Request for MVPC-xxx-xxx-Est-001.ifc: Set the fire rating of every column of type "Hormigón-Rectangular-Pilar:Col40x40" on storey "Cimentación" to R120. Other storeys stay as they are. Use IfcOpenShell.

First a look at what the model holds.

```python
import ifcopenshell
import ifcopenshell.util.element

model = ifcopenshell.open("MVPC-xxx-xxx-Est-001.ifc")
print(model.schema)
storey = next(s for s in model.by_type("IfcBuildingStorey") if s.Name == "Cimentación")
columns = [e for e in ifcopenshell.util.element.get_decomposition(storey) if e.is_a("IfcColumn")]
seen = {}
for e in columns:
    element_type = ifcopenshell.util.element.get_type(e)
    key = (element_type.Name if element_type != e and element_type else None, ifcopenshell.util.element.get_pset(e, "Pset_ColumnCommon", "FireRating"))
    seen[key] = seen.get(key, 0) + 1
for (name, value), count in sorted(seen.items(), key=str):
    print(count, "x", name, "|", value)
```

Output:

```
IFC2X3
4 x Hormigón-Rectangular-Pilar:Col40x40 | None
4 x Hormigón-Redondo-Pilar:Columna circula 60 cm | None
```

```python
import ifcopenshell
import ifcopenshell.api.pset
import ifcopenshell.util.element

model = ifcopenshell.open("MVPC-xxx-xxx-Est-001.ifc")

storey = next(s for s in model.by_type("IfcBuildingStorey") if s.Name == "Cimentación")
columns = [e for e in ifcopenshell.util.element.get_decomposition(storey) if e.is_a("IfcColumn")]

count = 0
for e in columns:
    element_type = ifcopenshell.util.element.get_type(e)
    if element_type in (None, e) or element_type.Name != "Hormigón-Rectangular-Pilar:Col40x40":
        continue
    # add_pset returns the element's existing set when there is one.
    pset = ifcopenshell.api.pset.add_pset(model, product=e, name="Pset_ColumnCommon")
    ifcopenshell.api.pset.edit_pset(model, pset=pset, properties={"FireRating": "R120"})
    count += 1

print(count, "columns updated")

model.write("MVPC-xxx-xxx-Est-001_rev.ifc")
```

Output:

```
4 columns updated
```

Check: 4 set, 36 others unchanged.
